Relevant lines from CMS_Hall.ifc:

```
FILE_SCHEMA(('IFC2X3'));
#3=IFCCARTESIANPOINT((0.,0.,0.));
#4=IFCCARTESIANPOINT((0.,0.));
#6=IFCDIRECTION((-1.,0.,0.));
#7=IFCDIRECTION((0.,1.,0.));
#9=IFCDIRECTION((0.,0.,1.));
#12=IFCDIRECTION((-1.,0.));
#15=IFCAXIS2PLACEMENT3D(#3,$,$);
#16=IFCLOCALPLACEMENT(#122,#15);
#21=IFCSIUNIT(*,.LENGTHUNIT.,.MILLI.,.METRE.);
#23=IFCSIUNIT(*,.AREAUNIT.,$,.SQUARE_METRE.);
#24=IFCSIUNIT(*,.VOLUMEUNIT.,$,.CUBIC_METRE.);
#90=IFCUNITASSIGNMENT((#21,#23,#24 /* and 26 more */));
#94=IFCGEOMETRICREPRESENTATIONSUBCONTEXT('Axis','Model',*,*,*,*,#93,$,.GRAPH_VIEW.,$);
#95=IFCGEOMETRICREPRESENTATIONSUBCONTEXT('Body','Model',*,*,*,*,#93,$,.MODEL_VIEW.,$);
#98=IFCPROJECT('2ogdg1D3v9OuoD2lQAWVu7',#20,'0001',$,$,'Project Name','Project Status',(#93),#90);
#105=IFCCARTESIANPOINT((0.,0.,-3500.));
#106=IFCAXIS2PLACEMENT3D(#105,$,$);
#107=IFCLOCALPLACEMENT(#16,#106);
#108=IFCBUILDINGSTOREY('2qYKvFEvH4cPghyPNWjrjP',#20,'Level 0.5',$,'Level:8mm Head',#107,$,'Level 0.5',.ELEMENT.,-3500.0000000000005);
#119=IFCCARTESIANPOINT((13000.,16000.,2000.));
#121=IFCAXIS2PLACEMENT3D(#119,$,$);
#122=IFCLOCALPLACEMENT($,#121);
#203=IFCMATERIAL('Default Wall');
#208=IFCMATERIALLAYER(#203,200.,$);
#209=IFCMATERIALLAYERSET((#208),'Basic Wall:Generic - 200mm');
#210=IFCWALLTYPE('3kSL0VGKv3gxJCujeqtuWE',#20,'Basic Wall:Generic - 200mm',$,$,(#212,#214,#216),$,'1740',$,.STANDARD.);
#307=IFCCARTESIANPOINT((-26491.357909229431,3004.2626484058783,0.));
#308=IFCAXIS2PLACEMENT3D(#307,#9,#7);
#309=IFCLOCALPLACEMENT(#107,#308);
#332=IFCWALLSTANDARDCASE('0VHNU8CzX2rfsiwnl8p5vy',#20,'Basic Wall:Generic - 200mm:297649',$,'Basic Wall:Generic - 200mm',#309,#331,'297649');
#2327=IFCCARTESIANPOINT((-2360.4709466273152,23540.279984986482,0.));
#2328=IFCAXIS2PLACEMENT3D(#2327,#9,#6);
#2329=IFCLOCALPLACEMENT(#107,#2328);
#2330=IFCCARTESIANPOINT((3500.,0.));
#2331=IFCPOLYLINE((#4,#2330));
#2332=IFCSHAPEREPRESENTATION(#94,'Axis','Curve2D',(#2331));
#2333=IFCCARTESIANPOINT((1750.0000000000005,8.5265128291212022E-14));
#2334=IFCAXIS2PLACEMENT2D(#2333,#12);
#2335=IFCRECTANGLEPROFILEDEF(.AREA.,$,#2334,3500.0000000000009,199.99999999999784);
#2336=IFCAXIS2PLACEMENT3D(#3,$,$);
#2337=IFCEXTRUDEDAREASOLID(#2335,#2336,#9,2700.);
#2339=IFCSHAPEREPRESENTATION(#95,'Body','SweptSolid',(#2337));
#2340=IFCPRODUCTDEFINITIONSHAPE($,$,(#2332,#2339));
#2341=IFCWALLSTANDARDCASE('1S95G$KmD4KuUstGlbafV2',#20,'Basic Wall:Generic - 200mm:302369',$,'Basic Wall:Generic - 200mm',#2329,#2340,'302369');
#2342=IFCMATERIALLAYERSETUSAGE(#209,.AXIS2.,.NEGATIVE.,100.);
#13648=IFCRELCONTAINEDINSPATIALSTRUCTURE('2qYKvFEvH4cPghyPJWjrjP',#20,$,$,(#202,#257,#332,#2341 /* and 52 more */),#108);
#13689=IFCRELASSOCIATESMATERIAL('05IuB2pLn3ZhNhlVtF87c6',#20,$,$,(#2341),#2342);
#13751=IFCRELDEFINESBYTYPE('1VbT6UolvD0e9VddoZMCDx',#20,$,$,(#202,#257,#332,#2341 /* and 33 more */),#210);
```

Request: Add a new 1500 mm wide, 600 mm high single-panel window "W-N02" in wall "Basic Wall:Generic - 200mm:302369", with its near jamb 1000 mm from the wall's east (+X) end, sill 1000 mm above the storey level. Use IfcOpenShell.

```python
import numpy as np
import ifcopenshell
import ifcopenshell.api.feature
import ifcopenshell.api.geometry
import ifcopenshell.api.root
import ifcopenshell.api.spatial
import ifcopenshell.api.type
import ifcopenshell.geom
import ifcopenshell.util.element
import ifcopenshell.util.placement
import ifcopenshell.util.representation
import ifcopenshell.util.shape
import ifcopenshell.util.unit

model = ifcopenshell.open("CMS_Hall.ifc")
unit_scale = ifcopenshell.util.unit.calculate_unit_scale(model)
settings = ifcopenshell.geom.settings()


def volume(element):
    """Net volume in cubic metres, openings subtracted."""
    shape = ifcopenshell.geom.create_shape(settings, element)
    return ifcopenshell.util.shape.get_volume(shape.geometry)


wall = model.by_guid("1S95G$KmD4KuUstGlbafV2")
storey = ifcopenshell.util.element.get_container(wall, ifc_class="IfcBuildingStorey")
context = ifcopenshell.util.representation.get_context(model, "Model", "Body", "MODEL_VIEW")
before = volume(wall)

width, height, from_end, sill = 1.5, 0.6, 1, 1  # metres

# The wall runs along its own X axis, and the end named is its -X end.
wall_shape = ifcopenshell.geom.create_shape(settings, wall)
x, y, z = ifcopenshell.util.shape.get_vertices(wall_shape.geometry).T
start = x.min() + from_end
face, thickness = float(y.min()), float(y.max() - y.min())
wall_matrix = ifcopenshell.util.placement.get_local_placement(wall.ObjectPlacement)
level = ifcopenshell.util.placement.get_local_placement(storey.ObjectPlacement)[2, 3]


def in_wall(x, y):
    """Placement at x, y metres in the wall's axes, at sill height."""
    matrix = wall_matrix.copy()
    matrix[:, 3] = wall_matrix @ np.array([x / unit_scale, y / unit_scale, 0.0, 1.0])
    matrix[2, 3] = level + sill / unit_scale
    return matrix


# Opening: a box that overshoots both wall faces by 50 mm.
opening = ifcopenshell.api.root.create_entity(model, ifc_class="IfcOpeningElement")
box = ifcopenshell.api.geometry.add_wall_representation(
    model, context=context, length=width, height=height, thickness=thickness + 0.1
)
ifcopenshell.api.geometry.assign_representation(model, product=opening, representation=box)
ifcopenshell.api.geometry.edit_object_placement(model, product=opening, matrix=in_wall(start, face - 0.05), is_si=False)
ifcopenshell.api.feature.add_feature(model, feature=opening, element=wall)

window = ifcopenshell.api.root.create_entity(model, ifc_class="IfcWindow", name="W-N02")
window.OverallWidth, window.OverallHeight = width / unit_scale, height / unit_scale
body = ifcopenshell.api.geometry.add_window_representation(
    model,
    context=context,
    overall_width=window.OverallWidth,
    overall_height=window.OverallHeight,
    partition_type="SINGLE_PANEL",
)
ifcopenshell.api.geometry.assign_representation(model, product=window, representation=body)
ifcopenshell.api.spatial.assign_container(model, products=[window], relating_structure=storey)
fills = ifcopenshell.api.feature.add_filling(model, opening=opening, element=window)
fills.OwnerHistory = window.OwnerHistory  # required in IFC2X3

# IFC2X3 keeps the operation on the window style.
style = ifcopenshell.api.root.create_entity(model, ifc_class="IfcWindowStyle", name="W-N02")
style.OperationType, style.ConstructionType = "SINGLE_PANEL", "NOTDEFINED"
style.ParameterTakesPrecedence = style.Sizeable = False
ifcopenshell.api.type.assign_type(model, related_objects=[window], relating_type=style)

# Centre the window in the wall's thickness.
ifcopenshell.api.geometry.edit_object_placement(model, product=window, matrix=in_wall(start, face), is_si=False)
window_shape = ifcopenshell.geom.create_shape(settings, window)
depth = ifcopenshell.util.shape.get_vertices(window_shape.geometry)[:, 1]
offset = face + thickness / 2 - (depth.min() + depth.max()) / 2
ifcopenshell.api.geometry.edit_object_placement(model, product=window, matrix=in_wall(start, offset), is_si=False)

after = volume(wall)

print(f"wall volume {before:.3f} -> {after:.3f} m3")

model.write("CMS_Hall_updated.ifc")
```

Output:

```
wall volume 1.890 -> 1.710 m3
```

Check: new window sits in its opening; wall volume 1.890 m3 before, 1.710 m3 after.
